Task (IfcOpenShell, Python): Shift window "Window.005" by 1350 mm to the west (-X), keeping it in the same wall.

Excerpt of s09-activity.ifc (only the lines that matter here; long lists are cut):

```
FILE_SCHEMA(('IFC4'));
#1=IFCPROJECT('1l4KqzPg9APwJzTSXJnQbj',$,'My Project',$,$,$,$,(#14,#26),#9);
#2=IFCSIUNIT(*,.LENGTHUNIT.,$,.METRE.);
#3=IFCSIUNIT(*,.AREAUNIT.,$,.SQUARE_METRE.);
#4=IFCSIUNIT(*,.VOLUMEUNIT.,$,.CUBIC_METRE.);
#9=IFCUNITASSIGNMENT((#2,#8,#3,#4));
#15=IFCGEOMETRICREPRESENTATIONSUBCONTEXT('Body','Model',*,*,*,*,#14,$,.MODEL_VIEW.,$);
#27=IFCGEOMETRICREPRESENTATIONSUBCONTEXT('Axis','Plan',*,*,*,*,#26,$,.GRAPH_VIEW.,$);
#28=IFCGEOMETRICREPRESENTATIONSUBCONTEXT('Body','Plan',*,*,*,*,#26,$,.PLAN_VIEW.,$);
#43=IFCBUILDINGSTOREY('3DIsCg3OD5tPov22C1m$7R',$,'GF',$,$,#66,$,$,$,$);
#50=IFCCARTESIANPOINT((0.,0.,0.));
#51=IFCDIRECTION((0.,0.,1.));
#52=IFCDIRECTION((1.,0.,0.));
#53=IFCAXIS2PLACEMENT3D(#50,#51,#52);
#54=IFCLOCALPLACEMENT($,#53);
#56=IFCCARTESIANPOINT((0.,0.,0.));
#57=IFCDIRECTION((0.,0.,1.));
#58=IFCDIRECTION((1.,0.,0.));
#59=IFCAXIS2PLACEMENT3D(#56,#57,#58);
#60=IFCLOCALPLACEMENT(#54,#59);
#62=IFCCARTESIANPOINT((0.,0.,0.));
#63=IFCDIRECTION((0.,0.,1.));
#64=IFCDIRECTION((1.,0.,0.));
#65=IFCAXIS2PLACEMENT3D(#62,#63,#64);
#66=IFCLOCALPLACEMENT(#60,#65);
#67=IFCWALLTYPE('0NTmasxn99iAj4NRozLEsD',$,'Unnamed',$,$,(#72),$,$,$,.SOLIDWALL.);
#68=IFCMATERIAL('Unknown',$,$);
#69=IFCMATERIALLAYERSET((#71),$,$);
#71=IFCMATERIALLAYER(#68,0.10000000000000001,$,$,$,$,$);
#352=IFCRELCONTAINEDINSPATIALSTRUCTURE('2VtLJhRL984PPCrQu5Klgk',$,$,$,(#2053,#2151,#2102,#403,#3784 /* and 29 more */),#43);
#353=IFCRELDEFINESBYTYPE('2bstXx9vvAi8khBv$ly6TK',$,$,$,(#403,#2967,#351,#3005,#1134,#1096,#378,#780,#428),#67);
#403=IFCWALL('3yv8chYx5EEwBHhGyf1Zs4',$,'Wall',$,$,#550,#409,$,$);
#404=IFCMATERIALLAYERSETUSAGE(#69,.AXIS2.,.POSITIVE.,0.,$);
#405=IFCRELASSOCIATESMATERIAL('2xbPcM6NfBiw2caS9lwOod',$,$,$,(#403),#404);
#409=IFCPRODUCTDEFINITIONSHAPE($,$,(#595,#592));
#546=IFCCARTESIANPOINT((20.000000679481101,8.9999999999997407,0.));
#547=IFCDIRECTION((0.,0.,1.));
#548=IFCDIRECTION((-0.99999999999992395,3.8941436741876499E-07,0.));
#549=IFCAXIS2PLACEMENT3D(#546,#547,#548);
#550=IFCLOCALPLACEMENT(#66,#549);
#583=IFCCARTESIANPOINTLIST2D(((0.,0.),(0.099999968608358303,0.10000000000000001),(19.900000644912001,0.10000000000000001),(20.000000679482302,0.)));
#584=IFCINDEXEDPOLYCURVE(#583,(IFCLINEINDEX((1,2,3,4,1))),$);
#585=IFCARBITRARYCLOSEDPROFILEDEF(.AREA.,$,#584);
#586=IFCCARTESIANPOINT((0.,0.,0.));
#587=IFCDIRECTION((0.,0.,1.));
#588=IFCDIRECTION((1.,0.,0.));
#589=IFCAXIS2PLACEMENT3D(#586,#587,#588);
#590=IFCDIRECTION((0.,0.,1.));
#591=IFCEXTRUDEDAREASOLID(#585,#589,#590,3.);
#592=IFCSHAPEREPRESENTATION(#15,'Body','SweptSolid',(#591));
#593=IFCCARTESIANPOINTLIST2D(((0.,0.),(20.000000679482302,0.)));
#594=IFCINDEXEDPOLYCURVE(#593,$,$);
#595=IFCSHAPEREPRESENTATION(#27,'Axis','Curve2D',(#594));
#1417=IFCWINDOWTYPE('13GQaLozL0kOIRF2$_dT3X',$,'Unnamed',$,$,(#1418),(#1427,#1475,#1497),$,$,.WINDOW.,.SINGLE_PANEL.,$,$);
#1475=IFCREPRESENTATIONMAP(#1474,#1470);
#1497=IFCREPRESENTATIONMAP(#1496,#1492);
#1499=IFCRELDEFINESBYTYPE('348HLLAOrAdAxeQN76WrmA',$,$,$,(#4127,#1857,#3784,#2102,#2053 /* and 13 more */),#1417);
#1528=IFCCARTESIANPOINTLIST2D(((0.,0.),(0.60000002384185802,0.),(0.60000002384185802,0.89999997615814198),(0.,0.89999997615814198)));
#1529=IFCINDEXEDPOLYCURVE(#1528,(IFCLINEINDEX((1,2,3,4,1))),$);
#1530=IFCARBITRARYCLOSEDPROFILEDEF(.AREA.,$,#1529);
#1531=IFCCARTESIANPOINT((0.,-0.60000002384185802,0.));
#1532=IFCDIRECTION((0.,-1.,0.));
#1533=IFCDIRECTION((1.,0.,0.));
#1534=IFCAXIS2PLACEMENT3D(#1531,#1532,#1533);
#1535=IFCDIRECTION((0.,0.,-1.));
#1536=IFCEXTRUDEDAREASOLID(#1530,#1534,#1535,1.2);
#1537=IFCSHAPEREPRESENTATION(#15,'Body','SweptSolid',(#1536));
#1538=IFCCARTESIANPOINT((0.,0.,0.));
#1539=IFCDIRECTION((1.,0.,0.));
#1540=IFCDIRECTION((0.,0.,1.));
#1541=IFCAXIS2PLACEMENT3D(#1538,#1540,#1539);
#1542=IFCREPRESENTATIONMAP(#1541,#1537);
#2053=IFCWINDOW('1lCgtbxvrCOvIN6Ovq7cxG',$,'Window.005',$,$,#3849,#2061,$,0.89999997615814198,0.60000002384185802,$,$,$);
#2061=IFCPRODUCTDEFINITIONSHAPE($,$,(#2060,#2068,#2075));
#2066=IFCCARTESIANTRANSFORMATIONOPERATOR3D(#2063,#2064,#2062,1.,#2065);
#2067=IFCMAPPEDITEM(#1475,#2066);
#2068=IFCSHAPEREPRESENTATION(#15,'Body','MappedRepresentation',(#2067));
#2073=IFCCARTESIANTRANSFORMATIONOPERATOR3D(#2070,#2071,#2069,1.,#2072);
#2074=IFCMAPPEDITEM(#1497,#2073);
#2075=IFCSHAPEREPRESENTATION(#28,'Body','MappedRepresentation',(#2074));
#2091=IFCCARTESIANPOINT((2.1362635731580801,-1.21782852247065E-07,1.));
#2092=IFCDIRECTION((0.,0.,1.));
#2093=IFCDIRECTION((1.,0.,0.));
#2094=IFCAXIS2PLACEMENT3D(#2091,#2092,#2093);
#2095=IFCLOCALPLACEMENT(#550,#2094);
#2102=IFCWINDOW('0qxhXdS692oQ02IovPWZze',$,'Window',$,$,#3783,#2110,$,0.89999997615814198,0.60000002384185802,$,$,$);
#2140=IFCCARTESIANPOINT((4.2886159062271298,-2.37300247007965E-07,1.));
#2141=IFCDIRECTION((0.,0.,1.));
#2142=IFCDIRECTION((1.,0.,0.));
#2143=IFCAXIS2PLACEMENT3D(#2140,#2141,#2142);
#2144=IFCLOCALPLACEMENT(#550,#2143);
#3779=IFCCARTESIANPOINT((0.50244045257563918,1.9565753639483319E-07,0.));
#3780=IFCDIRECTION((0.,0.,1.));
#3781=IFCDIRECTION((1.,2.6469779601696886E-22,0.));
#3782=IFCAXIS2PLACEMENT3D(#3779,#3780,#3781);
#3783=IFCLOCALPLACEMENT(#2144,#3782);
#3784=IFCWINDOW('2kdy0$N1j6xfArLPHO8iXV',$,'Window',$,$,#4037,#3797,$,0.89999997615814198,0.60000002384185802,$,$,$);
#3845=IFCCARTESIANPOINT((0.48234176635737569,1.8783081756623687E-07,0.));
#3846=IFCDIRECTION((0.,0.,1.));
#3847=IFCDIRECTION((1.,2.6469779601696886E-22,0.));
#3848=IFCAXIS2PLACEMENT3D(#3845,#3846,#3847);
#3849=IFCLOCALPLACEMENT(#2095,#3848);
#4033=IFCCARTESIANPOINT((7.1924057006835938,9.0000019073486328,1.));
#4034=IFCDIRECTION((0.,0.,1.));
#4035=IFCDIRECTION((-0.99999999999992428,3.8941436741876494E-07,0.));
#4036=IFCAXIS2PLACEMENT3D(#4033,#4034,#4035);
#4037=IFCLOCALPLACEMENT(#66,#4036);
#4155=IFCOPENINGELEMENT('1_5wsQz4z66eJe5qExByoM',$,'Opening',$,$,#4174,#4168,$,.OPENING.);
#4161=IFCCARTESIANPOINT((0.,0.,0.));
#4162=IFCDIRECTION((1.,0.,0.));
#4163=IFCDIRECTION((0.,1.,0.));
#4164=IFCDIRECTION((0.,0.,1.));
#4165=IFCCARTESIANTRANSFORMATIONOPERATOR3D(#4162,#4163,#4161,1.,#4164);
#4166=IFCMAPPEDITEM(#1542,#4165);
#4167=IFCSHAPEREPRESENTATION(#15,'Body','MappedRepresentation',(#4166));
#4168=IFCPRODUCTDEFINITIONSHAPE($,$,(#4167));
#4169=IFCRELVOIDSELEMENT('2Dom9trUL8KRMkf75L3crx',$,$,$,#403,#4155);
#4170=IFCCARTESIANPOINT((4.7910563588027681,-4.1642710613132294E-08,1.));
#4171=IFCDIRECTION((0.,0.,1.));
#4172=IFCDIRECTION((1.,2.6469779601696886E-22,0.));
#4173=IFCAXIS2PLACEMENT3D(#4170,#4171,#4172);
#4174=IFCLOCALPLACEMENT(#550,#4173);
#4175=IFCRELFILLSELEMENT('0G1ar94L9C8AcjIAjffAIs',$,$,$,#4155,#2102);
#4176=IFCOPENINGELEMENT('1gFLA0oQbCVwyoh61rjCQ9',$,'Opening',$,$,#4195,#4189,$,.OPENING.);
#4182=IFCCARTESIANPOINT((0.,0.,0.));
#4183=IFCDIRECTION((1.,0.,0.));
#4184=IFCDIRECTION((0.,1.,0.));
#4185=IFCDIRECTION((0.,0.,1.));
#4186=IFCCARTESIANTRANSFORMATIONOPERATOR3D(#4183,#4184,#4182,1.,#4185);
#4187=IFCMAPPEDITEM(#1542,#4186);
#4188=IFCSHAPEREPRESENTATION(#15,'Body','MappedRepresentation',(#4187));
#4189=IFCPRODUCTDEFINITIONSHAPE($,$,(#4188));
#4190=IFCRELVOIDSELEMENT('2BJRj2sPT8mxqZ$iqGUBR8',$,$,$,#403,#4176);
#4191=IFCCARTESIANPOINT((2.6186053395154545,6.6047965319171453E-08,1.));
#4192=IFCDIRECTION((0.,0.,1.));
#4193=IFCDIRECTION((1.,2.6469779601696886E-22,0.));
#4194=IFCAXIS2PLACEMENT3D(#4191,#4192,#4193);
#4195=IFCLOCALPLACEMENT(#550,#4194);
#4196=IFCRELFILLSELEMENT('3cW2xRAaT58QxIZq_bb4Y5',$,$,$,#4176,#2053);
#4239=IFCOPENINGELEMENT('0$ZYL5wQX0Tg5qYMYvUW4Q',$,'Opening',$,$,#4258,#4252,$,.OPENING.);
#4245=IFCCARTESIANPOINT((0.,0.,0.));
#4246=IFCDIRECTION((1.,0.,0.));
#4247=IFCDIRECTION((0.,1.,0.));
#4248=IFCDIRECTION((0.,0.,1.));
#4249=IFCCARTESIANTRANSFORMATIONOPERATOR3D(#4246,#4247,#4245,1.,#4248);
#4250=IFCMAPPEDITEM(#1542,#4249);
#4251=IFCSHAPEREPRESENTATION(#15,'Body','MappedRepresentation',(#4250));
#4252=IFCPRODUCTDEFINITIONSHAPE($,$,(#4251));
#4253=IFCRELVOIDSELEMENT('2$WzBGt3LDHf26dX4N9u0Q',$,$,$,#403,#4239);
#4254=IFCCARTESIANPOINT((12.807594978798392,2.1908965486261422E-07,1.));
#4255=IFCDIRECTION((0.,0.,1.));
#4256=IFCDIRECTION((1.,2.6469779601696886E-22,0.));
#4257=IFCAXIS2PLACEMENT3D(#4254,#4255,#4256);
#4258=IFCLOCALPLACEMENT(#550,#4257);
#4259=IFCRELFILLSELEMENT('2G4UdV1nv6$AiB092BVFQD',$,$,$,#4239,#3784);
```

```python
import ifcopenshell
import ifcopenshell.api.geometry
import ifcopenshell.util.placement
import ifcopenshell.util.unit

model = ifcopenshell.open("s09-activity.ifc")
unit_scale = ifcopenshell.util.unit.calculate_unit_scale(model)

window = model.by_guid("1lCgtbxvrCOvIN6Ovq7cxG")
opening = window.FillsVoids[0].RelatingOpeningElement
wall = opening.VoidsElements[0].RelatingBuildingElement

wall_matrix = ifcopenshell.util.placement.get_local_placement(wall.ObjectPlacement)
shift = wall_matrix[:3, 0] * 1.35 / unit_scale
before = ifcopenshell.util.placement.get_local_placement(window.ObjectPlacement)[:3, 3].copy()

# The window is not placed relative to its opening, so move both.
for product in (opening, window):
    matrix = ifcopenshell.util.placement.get_local_placement(product.ObjectPlacement)
    matrix[:3, 3] += shift
    ifcopenshell.api.geometry.edit_object_placement(model, product=product, matrix=matrix, is_si=False)

after = ifcopenshell.util.placement.get_local_placement(window.ObjectPlacement)[:3, 3]
print("window moved by", (after - before).round(3) + 0.0)

model.write("s09-activity_updated.ifc")
```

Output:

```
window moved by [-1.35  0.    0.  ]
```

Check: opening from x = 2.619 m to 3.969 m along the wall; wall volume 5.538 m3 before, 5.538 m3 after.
